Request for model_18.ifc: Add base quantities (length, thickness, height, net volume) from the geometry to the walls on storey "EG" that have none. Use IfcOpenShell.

First a look at what the model holds.

```python
import ifcopenshell
import ifcopenshell.util.element
import ifcopenshell.util.unit

model = ifcopenshell.open("model_18.ifc")
print(model.schema)
for unit_type in ("LENGTHUNIT", "AREAUNIT", "VOLUMEUNIT"):
    print(unit_type, ifcopenshell.util.unit.calculate_unit_scale(model, unit_type))
storey = next(s for s in model.by_type("IfcBuildingStorey") if s.Name == "EG")
walls = [e for e in ifcopenshell.util.element.get_decomposition(storey) if e.is_a("IfcWall")]
for e in sorted(walls, key=lambda e: e.id()):
    print(e.id(), e.is_a(), e.Name, list(ifcopenshell.util.element.get_psets(e, qtos_only=True)), sep=" | ")
```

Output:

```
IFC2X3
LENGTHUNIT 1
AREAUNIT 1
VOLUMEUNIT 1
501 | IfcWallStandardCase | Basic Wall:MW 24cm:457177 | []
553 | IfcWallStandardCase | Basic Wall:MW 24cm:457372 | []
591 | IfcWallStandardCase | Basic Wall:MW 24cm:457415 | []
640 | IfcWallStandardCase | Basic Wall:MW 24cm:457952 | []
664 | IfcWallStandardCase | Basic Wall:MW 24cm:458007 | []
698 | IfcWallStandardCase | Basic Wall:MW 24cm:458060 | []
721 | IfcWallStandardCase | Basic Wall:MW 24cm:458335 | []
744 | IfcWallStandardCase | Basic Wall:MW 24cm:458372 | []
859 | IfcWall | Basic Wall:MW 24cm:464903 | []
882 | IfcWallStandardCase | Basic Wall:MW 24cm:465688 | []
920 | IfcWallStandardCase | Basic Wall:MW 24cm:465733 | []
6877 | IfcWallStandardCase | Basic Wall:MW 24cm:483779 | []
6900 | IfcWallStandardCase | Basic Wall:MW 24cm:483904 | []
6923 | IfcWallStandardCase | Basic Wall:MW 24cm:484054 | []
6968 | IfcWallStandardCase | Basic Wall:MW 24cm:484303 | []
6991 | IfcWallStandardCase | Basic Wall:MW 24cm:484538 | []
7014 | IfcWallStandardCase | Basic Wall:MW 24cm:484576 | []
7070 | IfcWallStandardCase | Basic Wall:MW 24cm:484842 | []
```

```python
import ifcopenshell
import ifcopenshell.api.pset
import ifcopenshell.geom
import ifcopenshell.util.element
import ifcopenshell.util.shape
import ifcopenshell.util.unit

model = ifcopenshell.open("model_18.ifc")
unit_scale = ifcopenshell.util.unit.calculate_unit_scale(model)
volume_scale = ifcopenshell.util.unit.calculate_unit_scale(model, "VOLUMEUNIT")
settings = ifcopenshell.geom.settings()

storey = next(s for s in model.by_type("IfcBuildingStorey") if s.Name == "EG")
walls = [e for e in ifcopenshell.util.element.get_decomposition(storey) if e.is_a("IfcWall")]

for e in sorted(walls, key=lambda e: e.id()):
    if ifcopenshell.util.element.get_psets(e, qtos_only=True, should_inherit=False):
        continue
    # Geometry comes back in metres, in the element's own axes.
    shape = ifcopenshell.geom.create_shape(settings, e)
    values = {
        "Length": ifcopenshell.util.shape.get_x(shape.geometry) / unit_scale,
        "Width": ifcopenshell.util.shape.get_y(shape.geometry) / unit_scale,
        "Height": ifcopenshell.util.shape.get_z(shape.geometry) / unit_scale,
        "NetVolume": ifcopenshell.util.shape.get_volume(shape.geometry) / volume_scale,
    }
    qto = ifcopenshell.api.pset.add_qto(model, product=e, name="BaseQuantities")
    ifcopenshell.api.pset.edit_qto(model, qto=qto, properties=values)
    print(e.id(), {k: round(v, 3) for k, v in values.items()})

model.write("model_18-out.ifc")
```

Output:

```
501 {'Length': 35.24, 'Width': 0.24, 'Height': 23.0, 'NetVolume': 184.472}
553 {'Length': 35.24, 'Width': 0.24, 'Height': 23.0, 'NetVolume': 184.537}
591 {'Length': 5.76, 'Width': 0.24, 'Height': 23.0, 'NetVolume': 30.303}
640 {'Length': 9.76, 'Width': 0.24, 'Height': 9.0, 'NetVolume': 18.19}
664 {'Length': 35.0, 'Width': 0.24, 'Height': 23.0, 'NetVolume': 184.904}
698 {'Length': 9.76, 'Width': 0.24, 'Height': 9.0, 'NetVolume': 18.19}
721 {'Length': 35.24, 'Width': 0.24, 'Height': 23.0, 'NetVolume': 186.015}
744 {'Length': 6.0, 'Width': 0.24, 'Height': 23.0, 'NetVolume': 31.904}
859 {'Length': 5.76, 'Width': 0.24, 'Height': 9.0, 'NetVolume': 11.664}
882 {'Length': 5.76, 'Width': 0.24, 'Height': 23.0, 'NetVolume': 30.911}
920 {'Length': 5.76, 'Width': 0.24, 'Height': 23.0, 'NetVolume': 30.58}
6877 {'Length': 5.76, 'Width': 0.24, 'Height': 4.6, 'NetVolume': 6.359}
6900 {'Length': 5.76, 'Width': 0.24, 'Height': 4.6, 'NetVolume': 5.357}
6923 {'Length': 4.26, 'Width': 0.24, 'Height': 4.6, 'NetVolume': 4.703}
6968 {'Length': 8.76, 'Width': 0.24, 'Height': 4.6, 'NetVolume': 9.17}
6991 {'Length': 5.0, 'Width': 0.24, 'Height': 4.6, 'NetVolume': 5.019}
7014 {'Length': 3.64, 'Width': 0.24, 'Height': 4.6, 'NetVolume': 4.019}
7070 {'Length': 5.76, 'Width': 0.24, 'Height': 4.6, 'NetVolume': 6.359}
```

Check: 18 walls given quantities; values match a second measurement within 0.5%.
